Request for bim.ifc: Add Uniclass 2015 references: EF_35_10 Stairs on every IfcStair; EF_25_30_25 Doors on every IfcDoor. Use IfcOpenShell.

First a look at what the model holds.

```python
import ifcopenshell

model = ifcopenshell.open("bim.ifc")
print(model.schema)
print("classifications:", [c.Name for c in model.by_type("IfcClassification")])
for ifc_class in ("IfcDoor", "IfcRoof", "IfcStair", "IfcWall", "IfcWindow"):
    print(ifc_class, len(model.by_type(ifc_class)))
```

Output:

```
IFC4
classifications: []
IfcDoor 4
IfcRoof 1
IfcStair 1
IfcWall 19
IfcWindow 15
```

```python
import ifcopenshell
import ifcopenshell.api.classification

model = ifcopenshell.open("bim.ifc")

system = ifcopenshell.api.classification.add_classification(model, classification="Uniclass 2015")

codes = {
    "IfcStair": ("EF_35_10", "Stairs"),
    "IfcDoor": ("EF_25_30_25", "Doors"),
}
for ifc_class, (code, name) in codes.items():
    products = model.by_type(ifc_class)
    ifcopenshell.api.classification.add_reference(
        model, products=products, classification=system, identification=code, name=name
    )
    print(code, len(products))

model.write("bim_rev.ifc")
```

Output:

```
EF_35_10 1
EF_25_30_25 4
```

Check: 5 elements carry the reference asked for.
